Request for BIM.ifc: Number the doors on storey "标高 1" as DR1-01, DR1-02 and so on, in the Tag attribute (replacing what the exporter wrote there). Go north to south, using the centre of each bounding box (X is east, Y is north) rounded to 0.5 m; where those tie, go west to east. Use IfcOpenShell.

First a look at what the model holds.

```python
import ifcopenshell
import ifcopenshell.util.element
import ifcopenshell.util.placement

model = ifcopenshell.open("BIM.ifc")
print(model.schema)
storey = next(s for s in model.by_type("IfcBuildingStorey") if s.Name == "标高 1")
doors = [e for e in ifcopenshell.util.element.get_decomposition(storey) if e.is_a("IfcDoor")]
for e in sorted(doors, key=lambda e: e.id()):
    origin = ifcopenshell.util.placement.get_local_placement(e.ObjectPlacement)[:3, 3]
    print(e.id(), e.Tag, e.Name, origin.round(2) + 0.0, sep=" | ")
```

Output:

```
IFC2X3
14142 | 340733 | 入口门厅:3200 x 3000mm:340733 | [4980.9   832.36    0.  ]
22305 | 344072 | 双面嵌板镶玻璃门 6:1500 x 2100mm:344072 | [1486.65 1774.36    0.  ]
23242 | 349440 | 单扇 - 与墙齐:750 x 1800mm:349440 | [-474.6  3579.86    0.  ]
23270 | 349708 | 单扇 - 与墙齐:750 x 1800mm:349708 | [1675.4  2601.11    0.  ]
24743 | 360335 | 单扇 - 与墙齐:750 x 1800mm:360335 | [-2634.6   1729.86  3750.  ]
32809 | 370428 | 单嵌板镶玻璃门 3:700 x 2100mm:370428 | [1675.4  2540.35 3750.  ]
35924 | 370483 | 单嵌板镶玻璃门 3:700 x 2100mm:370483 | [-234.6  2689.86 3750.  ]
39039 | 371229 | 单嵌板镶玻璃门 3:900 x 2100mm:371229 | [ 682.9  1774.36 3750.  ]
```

```python
import ifcopenshell
import ifcopenshell.geom
import ifcopenshell.util.element
import ifcopenshell.util.shape

model = ifcopenshell.open("BIM.ifc")
settings = ifcopenshell.geom.settings()
settings.set("use-world-coords", True)


def centre(element):
    shape = ifcopenshell.geom.create_shape(settings, element)
    return ifcopenshell.util.shape.get_bbox_centroid(shape.geometry)


storey = next(s for s in model.by_type("IfcBuildingStorey") if s.Name == "标高 1")
doors = [e for e in ifcopenshell.util.element.get_decomposition(storey) if e.is_a("IfcDoor")]

# Insertion points can sit at a corner or the storey origin, so sort by the geometry (in metres).
centres = {e: centre(e) for e in doors}
doors.sort(key=lambda e: (-round(centres[e][1] / 0.5), centres[e][0]))

for i, e in enumerate(doors, start=1):
    number = f"DR1-{i:02d}"
    e.Tag = number
    print(e.id(), number)

model.write("BIM_rev.ifc")
```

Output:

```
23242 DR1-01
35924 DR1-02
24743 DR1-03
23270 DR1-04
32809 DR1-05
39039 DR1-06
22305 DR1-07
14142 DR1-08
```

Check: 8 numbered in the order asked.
